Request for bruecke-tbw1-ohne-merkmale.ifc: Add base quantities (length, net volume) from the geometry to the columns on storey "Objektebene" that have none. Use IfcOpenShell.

First a look at what the model holds.

```python
import ifcopenshell
import ifcopenshell.util.element
import ifcopenshell.util.unit

model = ifcopenshell.open("bruecke-tbw1-ohne-merkmale.ifc")
print(model.schema)
for unit_type in ("LENGTHUNIT", "AREAUNIT", "VOLUMEUNIT"):
    print(unit_type, ifcopenshell.util.unit.calculate_unit_scale(model, unit_type))
storey = next(s for s in model.by_type("IfcBuildingStorey") if s.Name == "Objektebene")
columns = [e for e in ifcopenshell.util.element.get_decomposition(storey) if e.is_a("IfcColumn")]
for e in sorted(columns, key=lambda e: e.id()):
    print(e.id(), e.is_a(), e.Name, list(ifcopenshell.util.element.get_psets(e, qtos_only=True)), sep=" | ")
```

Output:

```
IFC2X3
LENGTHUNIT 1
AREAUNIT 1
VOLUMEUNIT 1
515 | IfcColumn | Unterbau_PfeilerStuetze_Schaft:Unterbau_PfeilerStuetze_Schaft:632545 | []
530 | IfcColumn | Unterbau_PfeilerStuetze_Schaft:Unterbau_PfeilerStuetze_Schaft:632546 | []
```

```python
import ifcopenshell
import ifcopenshell.api.pset
import ifcopenshell.geom
import ifcopenshell.util.element
import ifcopenshell.util.shape
import ifcopenshell.util.unit

model = ifcopenshell.open("bruecke-tbw1-ohne-merkmale.ifc")
unit_scale = ifcopenshell.util.unit.calculate_unit_scale(model)
volume_scale = ifcopenshell.util.unit.calculate_unit_scale(model, "VOLUMEUNIT")
settings = ifcopenshell.geom.settings()

storey = next(s for s in model.by_type("IfcBuildingStorey") if s.Name == "Objektebene")
columns = [e for e in ifcopenshell.util.element.get_decomposition(storey) if e.is_a("IfcColumn")]

for e in sorted(columns, key=lambda e: e.id()):
    if ifcopenshell.util.element.get_psets(e, qtos_only=True, should_inherit=False):
        continue
    # Geometry comes back in metres, in the element's own axes.
    shape = ifcopenshell.geom.create_shape(settings, e)
    values = {
        "Length": ifcopenshell.util.shape.get_z(shape.geometry) / unit_scale,
        "NetVolume": ifcopenshell.util.shape.get_volume(shape.geometry) / volume_scale,
    }
    qto = ifcopenshell.api.pset.add_qto(model, product=e, name="BaseQuantities")
    ifcopenshell.api.pset.edit_qto(model, qto=qto, properties=values)
    print(e.id(), {k: round(v, 3) for k, v in values.items()})

model.write("bruecke-tbw1-ohne-merkmale_updated.ifc")
```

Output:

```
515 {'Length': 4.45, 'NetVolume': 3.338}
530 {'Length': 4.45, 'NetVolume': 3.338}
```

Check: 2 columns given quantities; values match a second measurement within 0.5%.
